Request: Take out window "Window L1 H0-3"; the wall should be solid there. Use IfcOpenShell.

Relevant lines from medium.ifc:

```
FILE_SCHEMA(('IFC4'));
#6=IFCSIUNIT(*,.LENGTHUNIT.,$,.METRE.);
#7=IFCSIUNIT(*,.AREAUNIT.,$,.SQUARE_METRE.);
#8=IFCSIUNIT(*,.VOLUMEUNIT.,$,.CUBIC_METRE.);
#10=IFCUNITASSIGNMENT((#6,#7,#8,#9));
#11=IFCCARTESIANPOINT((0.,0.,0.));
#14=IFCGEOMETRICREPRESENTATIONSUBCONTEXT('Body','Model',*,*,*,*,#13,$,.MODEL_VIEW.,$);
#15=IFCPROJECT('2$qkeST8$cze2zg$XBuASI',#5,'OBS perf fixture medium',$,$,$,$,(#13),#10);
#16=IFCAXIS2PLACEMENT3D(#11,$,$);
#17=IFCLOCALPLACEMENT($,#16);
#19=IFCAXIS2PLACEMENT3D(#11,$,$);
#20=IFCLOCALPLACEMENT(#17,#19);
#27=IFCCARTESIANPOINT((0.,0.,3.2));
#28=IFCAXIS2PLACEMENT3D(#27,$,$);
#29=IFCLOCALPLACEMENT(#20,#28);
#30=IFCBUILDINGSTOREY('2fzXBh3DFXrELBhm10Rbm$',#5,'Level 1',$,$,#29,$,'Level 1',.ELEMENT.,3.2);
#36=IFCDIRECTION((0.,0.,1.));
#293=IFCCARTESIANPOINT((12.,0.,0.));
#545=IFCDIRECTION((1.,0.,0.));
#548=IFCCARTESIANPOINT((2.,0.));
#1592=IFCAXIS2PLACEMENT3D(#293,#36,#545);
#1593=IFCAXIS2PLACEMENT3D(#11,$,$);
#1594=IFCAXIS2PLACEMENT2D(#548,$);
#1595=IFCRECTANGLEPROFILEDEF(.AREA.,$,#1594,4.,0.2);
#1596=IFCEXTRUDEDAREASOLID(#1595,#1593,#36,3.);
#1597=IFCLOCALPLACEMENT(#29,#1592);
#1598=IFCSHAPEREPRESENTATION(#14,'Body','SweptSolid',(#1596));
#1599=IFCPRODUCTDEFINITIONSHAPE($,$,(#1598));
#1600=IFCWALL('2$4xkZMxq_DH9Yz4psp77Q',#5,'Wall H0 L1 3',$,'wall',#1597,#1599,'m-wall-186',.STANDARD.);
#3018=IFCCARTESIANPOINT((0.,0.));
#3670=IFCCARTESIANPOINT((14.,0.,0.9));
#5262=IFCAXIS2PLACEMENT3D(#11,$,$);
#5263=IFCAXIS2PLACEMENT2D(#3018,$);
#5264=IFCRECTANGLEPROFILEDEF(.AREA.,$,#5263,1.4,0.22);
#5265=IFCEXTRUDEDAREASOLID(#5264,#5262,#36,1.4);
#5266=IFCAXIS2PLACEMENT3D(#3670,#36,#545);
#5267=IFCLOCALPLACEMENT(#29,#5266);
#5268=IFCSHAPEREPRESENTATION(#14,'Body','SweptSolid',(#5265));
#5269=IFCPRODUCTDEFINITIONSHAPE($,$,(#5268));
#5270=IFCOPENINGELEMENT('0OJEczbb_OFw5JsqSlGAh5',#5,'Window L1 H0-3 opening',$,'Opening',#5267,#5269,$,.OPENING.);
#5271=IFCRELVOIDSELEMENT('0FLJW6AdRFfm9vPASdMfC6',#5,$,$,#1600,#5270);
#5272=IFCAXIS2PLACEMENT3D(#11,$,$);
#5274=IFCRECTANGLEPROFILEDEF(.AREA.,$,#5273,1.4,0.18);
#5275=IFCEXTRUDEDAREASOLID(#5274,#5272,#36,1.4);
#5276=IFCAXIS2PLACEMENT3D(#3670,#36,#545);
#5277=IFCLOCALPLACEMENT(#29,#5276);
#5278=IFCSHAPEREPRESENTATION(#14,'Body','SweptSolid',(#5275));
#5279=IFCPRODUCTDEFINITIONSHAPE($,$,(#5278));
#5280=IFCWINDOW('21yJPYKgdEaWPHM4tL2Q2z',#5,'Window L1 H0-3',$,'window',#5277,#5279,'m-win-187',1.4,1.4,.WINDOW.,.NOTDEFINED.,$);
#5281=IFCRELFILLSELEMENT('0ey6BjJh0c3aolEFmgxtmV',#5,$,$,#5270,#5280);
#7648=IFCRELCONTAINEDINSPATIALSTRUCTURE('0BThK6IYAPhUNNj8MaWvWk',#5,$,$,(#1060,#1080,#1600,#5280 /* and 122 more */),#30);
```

```python
import ifcopenshell
import ifcopenshell.api.feature
import ifcopenshell.api.root
import ifcopenshell.geom
import ifcopenshell.util.shape

model = ifcopenshell.open("medium.ifc")
settings = ifcopenshell.geom.settings()


def volume(element):
    """Net volume in cubic metres, openings subtracted."""
    shape = ifcopenshell.geom.create_shape(settings, element)
    return ifcopenshell.util.shape.get_volume(shape.geometry)


window = model.by_guid("21yJPYKgdEaWPHM4tL2Q2z")
opening = window.FillsVoids[0].RelatingOpeningElement
wall = opening.VoidsElements[0].RelatingBuildingElement
before = volume(wall)

ifcopenshell.api.root.remove_product(model, product=window)
ifcopenshell.api.feature.remove_feature(model, feature=opening)

after = volume(wall)

print(f"wall volume {before:.3f} -> {after:.3f} m3")

model.write("medium_v2.ifc")
```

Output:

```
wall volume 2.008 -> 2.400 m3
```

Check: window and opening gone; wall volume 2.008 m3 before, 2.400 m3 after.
